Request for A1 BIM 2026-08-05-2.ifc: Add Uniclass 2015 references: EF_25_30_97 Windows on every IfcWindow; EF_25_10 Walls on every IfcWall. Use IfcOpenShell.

First a look at what the model holds.

```python
import ifcopenshell

model = ifcopenshell.open("A1 BIM 2026-08-05-2.ifc")
print(model.schema)
print("classifications:", [c.Name for c in model.by_type("IfcClassification")])
for ifc_class in ("IfcDoor", "IfcRoof", "IfcStair", "IfcWall", "IfcWindow"):
    print(ifc_class, len(model.by_type(ifc_class)))
```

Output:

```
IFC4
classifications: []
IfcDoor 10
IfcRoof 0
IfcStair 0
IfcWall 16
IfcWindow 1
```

```python
import ifcopenshell
import ifcopenshell.api.classification

model = ifcopenshell.open("A1 BIM 2026-08-05-2.ifc")

system = ifcopenshell.api.classification.add_classification(model, classification="Uniclass 2015")

codes = {
    "IfcWindow": ("EF_25_30_97", "Windows"),
    "IfcWall": ("EF_25_10", "Walls"),
}
for ifc_class, (code, name) in codes.items():
    products = model.by_type(ifc_class)
    ifcopenshell.api.classification.add_reference(
        model, products=products, classification=system, identification=code, name=name
    )
    print(code, len(products))

model.write("A1 BIM 2026-08-05-2_edited.ifc")
```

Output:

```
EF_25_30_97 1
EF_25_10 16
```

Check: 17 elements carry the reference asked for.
